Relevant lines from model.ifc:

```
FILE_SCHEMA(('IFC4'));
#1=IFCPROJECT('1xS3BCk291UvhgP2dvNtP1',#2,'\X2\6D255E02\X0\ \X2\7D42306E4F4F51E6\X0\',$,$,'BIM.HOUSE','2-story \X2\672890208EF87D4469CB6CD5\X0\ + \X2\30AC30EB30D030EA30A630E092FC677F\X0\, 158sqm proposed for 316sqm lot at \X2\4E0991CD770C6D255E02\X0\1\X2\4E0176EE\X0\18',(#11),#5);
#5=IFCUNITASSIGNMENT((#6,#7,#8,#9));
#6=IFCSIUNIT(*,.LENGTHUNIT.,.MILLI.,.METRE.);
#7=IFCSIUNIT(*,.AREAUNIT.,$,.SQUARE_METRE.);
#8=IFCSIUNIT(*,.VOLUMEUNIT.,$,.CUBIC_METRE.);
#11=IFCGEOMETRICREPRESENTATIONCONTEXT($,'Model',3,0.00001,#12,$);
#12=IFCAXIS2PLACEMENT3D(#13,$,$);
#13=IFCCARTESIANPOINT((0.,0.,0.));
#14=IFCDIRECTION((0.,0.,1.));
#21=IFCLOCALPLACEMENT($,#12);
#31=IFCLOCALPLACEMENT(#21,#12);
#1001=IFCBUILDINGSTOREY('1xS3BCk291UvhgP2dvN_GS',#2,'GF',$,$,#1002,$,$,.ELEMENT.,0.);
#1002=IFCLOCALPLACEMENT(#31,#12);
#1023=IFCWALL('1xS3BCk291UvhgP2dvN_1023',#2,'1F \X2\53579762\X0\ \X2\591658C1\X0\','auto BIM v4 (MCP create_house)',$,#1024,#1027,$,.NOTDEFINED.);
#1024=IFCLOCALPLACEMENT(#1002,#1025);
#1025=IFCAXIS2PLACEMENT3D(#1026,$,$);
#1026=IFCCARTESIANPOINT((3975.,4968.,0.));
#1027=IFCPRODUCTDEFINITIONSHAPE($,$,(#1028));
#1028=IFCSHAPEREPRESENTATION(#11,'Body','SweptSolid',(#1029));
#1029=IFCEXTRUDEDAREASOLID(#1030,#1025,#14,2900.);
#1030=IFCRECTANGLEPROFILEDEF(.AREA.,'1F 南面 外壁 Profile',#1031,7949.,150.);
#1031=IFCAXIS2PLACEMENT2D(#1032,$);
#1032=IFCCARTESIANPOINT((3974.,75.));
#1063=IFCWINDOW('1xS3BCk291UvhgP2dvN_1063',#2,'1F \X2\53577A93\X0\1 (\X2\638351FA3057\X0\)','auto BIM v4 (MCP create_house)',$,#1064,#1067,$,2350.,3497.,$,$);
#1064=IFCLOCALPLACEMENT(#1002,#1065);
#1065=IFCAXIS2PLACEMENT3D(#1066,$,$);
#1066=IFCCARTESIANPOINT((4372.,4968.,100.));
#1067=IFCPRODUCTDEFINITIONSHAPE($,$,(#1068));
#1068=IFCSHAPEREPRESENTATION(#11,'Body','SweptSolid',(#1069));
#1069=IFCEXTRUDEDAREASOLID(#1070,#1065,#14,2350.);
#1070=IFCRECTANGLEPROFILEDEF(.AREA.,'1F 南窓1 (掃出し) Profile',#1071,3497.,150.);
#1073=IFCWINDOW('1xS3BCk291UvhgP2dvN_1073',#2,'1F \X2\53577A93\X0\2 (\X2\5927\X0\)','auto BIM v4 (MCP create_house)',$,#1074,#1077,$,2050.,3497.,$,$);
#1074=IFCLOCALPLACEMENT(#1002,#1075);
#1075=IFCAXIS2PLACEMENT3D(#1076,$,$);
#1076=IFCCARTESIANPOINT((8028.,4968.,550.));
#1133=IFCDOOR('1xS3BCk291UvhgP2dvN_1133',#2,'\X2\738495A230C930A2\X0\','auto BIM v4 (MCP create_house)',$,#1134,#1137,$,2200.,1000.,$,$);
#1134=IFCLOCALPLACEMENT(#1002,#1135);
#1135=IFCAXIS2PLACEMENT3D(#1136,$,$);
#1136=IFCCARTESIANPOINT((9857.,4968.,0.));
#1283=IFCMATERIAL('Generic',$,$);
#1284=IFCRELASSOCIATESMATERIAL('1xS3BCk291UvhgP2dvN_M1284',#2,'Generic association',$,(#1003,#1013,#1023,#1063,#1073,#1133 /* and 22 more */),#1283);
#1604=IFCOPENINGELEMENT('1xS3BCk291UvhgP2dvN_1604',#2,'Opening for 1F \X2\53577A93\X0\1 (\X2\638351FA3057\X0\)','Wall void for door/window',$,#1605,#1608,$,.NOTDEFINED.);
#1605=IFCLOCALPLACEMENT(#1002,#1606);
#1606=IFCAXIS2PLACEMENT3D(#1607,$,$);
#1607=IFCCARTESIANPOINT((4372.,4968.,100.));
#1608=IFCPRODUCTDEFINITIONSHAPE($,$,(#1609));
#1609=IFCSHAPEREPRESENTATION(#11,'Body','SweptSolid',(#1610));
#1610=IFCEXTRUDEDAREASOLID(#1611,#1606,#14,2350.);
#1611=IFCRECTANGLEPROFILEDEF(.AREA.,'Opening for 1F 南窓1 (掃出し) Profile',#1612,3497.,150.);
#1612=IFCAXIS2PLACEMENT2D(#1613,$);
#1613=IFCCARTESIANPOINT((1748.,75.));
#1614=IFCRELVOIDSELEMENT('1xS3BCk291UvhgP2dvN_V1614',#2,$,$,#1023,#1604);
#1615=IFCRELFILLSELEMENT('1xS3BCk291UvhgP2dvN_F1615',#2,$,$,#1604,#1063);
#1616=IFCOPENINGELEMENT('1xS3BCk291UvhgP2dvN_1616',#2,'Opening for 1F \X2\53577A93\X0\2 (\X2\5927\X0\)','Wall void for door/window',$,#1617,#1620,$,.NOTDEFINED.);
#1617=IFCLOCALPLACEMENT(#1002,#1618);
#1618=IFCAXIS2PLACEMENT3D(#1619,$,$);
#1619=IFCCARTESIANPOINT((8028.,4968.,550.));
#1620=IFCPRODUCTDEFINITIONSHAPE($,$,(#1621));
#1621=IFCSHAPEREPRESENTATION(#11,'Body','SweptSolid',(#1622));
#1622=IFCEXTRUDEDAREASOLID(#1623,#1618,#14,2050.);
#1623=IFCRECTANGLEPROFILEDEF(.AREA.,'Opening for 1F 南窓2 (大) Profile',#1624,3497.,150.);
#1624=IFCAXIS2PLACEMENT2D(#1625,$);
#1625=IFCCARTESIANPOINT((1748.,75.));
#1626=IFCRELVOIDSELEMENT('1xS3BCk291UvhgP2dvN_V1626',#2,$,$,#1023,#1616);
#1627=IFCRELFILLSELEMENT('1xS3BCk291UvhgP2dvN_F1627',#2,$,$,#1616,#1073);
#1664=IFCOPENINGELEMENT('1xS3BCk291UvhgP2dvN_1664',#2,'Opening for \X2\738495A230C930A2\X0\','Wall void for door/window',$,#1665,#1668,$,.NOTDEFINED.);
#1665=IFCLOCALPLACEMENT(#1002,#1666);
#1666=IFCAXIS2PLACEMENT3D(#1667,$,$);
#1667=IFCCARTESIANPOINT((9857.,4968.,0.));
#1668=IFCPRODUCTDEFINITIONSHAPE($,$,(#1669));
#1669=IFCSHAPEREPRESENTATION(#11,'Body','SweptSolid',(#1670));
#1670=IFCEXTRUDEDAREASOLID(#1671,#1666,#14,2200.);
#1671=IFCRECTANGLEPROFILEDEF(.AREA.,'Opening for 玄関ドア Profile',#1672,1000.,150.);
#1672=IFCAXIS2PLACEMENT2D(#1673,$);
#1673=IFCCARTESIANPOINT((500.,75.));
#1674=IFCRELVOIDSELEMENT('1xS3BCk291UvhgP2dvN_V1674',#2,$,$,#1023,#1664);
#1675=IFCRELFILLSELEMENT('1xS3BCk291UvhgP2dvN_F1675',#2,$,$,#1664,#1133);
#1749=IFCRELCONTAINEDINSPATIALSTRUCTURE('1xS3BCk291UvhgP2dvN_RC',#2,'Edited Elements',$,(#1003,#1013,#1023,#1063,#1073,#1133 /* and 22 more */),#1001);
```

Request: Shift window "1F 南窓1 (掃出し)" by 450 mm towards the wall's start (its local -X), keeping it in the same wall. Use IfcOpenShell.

```python
import ifcopenshell
import ifcopenshell.api.geometry
import ifcopenshell.util.placement

model = ifcopenshell.open("model.ifc")

window = model.by_guid("1xS3BCk291UvhgP2dvN_1063")
opening = window.FillsVoids[0].RelatingOpeningElement
wall = opening.VoidsElements[0].RelatingBuildingElement

wall_matrix = ifcopenshell.util.placement.get_local_placement(wall.ObjectPlacement)
shift = wall_matrix[:3, 0] * -450.0
before = ifcopenshell.util.placement.get_local_placement(window.ObjectPlacement)[:3, 3].copy()

# The window is not placed relative to its opening, so move both.
for product in (opening, window):
    matrix = ifcopenshell.util.placement.get_local_placement(product.ObjectPlacement)
    matrix[:3, 3] += shift
    ifcopenshell.api.geometry.edit_object_placement(model, product=product, matrix=matrix, is_si=False)

after = ifcopenshell.util.placement.get_local_placement(window.ObjectPlacement)[:3, 3]
print("window moved by", (after - before).round(3) + 0.0)

model.write("model-out.ifc")
```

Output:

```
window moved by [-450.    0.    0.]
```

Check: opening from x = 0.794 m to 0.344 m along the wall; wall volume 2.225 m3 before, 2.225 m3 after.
